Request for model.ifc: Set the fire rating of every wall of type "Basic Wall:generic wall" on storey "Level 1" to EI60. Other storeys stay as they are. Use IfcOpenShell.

First a look at what the model holds.

```python
import ifcopenshell
import ifcopenshell.util.element

model = ifcopenshell.open("model.ifc")
print(model.schema)
storey = next(s for s in model.by_type("IfcBuildingStorey") if s.Name == "Level 1")
walls = [e for e in ifcopenshell.util.element.get_decomposition(storey) if e.is_a("IfcWall")]
seen = {}
for e in walls:
    element_type = ifcopenshell.util.element.get_type(e)
    key = (element_type.Name if element_type != e and element_type else None, ifcopenshell.util.element.get_pset(e, "Pset_WallCommon", "FireRating"))
    seen[key] = seen.get(key, 0) + 1
for (name, value), count in sorted(seen.items(), key=str):
    print(count, "x", name, "|", value)
```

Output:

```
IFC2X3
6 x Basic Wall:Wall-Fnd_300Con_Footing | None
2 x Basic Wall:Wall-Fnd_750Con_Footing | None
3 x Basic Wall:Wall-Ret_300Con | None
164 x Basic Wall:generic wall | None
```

```python
import ifcopenshell
import ifcopenshell.api.pset
import ifcopenshell.util.element

model = ifcopenshell.open("model.ifc")

storey = next(s for s in model.by_type("IfcBuildingStorey") if s.Name == "Level 1")
walls = [e for e in ifcopenshell.util.element.get_decomposition(storey) if e.is_a("IfcWall")]

count = 0
for e in walls:
    element_type = ifcopenshell.util.element.get_type(e)
    if element_type in (None, e) or element_type.Name != "Basic Wall:generic wall":
        continue
    # add_pset returns the element's existing set when there is one.
    pset = ifcopenshell.api.pset.add_pset(model, product=e, name="Pset_WallCommon")
    ifcopenshell.api.pset.edit_pset(model, pset=pset, properties={"FireRating": "EI60"})
    count += 1

print(count, "walls updated")

model.write("model_updated.ifc")
```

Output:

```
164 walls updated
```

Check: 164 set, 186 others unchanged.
